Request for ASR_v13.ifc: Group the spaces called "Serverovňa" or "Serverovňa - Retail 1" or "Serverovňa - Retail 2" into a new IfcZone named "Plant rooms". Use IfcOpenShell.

First a look at what the model holds.

```python
import ifcopenshell

model = ifcopenshell.open("ASR_v13.ifc")
print(model.schema)
seen = {}
for space in model.by_type("IfcSpace"):
    seen[space.LongName] = seen.get(space.LongName, 0) + 1
for name, count in sorted(seen.items(), key=str):
    print(count, "x", name)
print("zones:", [z.Name for z in model.by_type("IfcZone")][:20])
```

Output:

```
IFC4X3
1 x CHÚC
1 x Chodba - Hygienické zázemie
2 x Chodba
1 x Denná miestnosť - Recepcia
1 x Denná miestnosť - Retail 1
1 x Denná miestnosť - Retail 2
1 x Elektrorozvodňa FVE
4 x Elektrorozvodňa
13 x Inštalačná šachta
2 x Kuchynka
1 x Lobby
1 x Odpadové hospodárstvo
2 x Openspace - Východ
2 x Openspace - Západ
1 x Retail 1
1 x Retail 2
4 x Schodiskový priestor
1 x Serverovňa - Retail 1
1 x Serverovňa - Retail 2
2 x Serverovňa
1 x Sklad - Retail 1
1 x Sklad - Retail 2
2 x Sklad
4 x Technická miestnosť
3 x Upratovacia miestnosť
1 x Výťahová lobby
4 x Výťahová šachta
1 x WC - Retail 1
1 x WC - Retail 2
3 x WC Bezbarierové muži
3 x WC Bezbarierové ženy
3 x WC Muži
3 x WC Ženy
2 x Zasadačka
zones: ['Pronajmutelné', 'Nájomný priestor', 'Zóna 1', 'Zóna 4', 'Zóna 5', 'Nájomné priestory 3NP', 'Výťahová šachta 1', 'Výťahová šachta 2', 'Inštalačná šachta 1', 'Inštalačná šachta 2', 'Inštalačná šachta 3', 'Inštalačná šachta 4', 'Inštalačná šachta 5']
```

```python
import ifcopenshell
import ifcopenshell.api.group
import ifcopenshell.api.root

model = ifcopenshell.open("ASR_v13.ifc")

names = {"Serverovňa", "Serverovňa - Retail 1", "Serverovňa - Retail 2"}
spaces = [s for s in model.by_type("IfcSpace") if s.LongName in names]

zone = ifcopenshell.api.root.create_entity(model, ifc_class="IfcZone", name="Plant rooms")
ifcopenshell.api.group.assign_group(model, products=spaces, group=zone)
print(len(spaces), "spaces in", zone.Name)

model.write("ASR_v13-out.ifc")
```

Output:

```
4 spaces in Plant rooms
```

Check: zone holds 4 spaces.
